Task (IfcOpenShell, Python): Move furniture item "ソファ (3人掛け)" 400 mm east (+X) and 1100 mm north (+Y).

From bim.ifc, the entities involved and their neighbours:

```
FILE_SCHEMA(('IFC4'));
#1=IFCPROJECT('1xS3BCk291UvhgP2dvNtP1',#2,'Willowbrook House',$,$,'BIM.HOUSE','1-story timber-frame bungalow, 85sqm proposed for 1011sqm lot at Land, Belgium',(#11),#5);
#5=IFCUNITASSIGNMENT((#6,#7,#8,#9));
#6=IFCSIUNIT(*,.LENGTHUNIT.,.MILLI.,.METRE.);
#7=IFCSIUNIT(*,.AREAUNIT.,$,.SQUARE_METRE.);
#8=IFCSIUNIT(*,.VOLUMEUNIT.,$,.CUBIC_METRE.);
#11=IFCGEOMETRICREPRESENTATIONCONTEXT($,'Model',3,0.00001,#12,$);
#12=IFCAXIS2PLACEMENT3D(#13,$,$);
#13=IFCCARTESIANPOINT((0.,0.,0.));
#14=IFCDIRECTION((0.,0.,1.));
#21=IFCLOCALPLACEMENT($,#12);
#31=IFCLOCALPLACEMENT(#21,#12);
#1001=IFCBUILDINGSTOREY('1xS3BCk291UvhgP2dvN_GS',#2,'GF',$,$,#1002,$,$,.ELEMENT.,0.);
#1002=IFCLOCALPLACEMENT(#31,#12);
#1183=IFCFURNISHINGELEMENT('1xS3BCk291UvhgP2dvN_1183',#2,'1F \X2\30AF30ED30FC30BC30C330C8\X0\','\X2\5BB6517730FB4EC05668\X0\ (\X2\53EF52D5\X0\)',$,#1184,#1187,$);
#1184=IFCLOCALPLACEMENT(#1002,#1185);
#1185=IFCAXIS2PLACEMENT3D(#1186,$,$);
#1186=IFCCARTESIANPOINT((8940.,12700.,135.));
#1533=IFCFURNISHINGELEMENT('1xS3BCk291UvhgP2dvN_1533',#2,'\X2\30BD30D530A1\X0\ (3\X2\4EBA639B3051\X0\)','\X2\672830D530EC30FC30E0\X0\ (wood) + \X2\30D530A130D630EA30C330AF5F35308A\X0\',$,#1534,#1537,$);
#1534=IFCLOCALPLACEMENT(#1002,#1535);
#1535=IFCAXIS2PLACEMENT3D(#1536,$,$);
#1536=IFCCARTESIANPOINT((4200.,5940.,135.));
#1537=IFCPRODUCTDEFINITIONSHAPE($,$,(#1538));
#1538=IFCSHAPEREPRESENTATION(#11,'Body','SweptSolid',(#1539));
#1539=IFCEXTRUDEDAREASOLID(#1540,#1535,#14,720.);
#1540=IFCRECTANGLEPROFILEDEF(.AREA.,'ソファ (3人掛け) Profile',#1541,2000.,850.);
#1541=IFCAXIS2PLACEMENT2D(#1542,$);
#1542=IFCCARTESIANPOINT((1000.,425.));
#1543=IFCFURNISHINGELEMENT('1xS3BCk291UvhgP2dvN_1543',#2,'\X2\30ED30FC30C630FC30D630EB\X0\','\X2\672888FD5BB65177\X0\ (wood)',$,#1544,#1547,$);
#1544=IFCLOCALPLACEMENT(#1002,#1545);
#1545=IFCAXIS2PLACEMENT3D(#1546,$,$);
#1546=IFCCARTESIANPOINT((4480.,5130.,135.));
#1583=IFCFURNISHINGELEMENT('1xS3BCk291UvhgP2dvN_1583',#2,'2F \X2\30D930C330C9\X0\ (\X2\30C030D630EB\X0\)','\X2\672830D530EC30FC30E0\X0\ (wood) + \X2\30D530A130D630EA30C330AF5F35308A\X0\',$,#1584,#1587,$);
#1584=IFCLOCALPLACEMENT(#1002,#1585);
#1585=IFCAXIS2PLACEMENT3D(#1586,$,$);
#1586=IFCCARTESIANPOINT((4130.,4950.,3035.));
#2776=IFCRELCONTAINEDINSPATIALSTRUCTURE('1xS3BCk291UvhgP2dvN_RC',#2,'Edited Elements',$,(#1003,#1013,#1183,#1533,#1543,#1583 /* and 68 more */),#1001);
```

```python
import ifcopenshell
import ifcopenshell.api.geometry
import ifcopenshell.util.placement
import ifcopenshell.util.unit

model = ifcopenshell.open("bim.ifc")
unit_scale = ifcopenshell.util.unit.calculate_unit_scale(model)

item = model.by_id(1533)
matrix = ifcopenshell.util.placement.get_local_placement(item.ObjectPlacement)
matrix[0, 3] += 0.4 / unit_scale
matrix[1, 3] += 1.1 / unit_scale
ifcopenshell.api.geometry.edit_object_placement(model, product=item, matrix=matrix, is_si=False)

print(ifcopenshell.util.placement.get_local_placement(item.ObjectPlacement).round(3) + 0.0)

model.write("bim-out.ifc")
```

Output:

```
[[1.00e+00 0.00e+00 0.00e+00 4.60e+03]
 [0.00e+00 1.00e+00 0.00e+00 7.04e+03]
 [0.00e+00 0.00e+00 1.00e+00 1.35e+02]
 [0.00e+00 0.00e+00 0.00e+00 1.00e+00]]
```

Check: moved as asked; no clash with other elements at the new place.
